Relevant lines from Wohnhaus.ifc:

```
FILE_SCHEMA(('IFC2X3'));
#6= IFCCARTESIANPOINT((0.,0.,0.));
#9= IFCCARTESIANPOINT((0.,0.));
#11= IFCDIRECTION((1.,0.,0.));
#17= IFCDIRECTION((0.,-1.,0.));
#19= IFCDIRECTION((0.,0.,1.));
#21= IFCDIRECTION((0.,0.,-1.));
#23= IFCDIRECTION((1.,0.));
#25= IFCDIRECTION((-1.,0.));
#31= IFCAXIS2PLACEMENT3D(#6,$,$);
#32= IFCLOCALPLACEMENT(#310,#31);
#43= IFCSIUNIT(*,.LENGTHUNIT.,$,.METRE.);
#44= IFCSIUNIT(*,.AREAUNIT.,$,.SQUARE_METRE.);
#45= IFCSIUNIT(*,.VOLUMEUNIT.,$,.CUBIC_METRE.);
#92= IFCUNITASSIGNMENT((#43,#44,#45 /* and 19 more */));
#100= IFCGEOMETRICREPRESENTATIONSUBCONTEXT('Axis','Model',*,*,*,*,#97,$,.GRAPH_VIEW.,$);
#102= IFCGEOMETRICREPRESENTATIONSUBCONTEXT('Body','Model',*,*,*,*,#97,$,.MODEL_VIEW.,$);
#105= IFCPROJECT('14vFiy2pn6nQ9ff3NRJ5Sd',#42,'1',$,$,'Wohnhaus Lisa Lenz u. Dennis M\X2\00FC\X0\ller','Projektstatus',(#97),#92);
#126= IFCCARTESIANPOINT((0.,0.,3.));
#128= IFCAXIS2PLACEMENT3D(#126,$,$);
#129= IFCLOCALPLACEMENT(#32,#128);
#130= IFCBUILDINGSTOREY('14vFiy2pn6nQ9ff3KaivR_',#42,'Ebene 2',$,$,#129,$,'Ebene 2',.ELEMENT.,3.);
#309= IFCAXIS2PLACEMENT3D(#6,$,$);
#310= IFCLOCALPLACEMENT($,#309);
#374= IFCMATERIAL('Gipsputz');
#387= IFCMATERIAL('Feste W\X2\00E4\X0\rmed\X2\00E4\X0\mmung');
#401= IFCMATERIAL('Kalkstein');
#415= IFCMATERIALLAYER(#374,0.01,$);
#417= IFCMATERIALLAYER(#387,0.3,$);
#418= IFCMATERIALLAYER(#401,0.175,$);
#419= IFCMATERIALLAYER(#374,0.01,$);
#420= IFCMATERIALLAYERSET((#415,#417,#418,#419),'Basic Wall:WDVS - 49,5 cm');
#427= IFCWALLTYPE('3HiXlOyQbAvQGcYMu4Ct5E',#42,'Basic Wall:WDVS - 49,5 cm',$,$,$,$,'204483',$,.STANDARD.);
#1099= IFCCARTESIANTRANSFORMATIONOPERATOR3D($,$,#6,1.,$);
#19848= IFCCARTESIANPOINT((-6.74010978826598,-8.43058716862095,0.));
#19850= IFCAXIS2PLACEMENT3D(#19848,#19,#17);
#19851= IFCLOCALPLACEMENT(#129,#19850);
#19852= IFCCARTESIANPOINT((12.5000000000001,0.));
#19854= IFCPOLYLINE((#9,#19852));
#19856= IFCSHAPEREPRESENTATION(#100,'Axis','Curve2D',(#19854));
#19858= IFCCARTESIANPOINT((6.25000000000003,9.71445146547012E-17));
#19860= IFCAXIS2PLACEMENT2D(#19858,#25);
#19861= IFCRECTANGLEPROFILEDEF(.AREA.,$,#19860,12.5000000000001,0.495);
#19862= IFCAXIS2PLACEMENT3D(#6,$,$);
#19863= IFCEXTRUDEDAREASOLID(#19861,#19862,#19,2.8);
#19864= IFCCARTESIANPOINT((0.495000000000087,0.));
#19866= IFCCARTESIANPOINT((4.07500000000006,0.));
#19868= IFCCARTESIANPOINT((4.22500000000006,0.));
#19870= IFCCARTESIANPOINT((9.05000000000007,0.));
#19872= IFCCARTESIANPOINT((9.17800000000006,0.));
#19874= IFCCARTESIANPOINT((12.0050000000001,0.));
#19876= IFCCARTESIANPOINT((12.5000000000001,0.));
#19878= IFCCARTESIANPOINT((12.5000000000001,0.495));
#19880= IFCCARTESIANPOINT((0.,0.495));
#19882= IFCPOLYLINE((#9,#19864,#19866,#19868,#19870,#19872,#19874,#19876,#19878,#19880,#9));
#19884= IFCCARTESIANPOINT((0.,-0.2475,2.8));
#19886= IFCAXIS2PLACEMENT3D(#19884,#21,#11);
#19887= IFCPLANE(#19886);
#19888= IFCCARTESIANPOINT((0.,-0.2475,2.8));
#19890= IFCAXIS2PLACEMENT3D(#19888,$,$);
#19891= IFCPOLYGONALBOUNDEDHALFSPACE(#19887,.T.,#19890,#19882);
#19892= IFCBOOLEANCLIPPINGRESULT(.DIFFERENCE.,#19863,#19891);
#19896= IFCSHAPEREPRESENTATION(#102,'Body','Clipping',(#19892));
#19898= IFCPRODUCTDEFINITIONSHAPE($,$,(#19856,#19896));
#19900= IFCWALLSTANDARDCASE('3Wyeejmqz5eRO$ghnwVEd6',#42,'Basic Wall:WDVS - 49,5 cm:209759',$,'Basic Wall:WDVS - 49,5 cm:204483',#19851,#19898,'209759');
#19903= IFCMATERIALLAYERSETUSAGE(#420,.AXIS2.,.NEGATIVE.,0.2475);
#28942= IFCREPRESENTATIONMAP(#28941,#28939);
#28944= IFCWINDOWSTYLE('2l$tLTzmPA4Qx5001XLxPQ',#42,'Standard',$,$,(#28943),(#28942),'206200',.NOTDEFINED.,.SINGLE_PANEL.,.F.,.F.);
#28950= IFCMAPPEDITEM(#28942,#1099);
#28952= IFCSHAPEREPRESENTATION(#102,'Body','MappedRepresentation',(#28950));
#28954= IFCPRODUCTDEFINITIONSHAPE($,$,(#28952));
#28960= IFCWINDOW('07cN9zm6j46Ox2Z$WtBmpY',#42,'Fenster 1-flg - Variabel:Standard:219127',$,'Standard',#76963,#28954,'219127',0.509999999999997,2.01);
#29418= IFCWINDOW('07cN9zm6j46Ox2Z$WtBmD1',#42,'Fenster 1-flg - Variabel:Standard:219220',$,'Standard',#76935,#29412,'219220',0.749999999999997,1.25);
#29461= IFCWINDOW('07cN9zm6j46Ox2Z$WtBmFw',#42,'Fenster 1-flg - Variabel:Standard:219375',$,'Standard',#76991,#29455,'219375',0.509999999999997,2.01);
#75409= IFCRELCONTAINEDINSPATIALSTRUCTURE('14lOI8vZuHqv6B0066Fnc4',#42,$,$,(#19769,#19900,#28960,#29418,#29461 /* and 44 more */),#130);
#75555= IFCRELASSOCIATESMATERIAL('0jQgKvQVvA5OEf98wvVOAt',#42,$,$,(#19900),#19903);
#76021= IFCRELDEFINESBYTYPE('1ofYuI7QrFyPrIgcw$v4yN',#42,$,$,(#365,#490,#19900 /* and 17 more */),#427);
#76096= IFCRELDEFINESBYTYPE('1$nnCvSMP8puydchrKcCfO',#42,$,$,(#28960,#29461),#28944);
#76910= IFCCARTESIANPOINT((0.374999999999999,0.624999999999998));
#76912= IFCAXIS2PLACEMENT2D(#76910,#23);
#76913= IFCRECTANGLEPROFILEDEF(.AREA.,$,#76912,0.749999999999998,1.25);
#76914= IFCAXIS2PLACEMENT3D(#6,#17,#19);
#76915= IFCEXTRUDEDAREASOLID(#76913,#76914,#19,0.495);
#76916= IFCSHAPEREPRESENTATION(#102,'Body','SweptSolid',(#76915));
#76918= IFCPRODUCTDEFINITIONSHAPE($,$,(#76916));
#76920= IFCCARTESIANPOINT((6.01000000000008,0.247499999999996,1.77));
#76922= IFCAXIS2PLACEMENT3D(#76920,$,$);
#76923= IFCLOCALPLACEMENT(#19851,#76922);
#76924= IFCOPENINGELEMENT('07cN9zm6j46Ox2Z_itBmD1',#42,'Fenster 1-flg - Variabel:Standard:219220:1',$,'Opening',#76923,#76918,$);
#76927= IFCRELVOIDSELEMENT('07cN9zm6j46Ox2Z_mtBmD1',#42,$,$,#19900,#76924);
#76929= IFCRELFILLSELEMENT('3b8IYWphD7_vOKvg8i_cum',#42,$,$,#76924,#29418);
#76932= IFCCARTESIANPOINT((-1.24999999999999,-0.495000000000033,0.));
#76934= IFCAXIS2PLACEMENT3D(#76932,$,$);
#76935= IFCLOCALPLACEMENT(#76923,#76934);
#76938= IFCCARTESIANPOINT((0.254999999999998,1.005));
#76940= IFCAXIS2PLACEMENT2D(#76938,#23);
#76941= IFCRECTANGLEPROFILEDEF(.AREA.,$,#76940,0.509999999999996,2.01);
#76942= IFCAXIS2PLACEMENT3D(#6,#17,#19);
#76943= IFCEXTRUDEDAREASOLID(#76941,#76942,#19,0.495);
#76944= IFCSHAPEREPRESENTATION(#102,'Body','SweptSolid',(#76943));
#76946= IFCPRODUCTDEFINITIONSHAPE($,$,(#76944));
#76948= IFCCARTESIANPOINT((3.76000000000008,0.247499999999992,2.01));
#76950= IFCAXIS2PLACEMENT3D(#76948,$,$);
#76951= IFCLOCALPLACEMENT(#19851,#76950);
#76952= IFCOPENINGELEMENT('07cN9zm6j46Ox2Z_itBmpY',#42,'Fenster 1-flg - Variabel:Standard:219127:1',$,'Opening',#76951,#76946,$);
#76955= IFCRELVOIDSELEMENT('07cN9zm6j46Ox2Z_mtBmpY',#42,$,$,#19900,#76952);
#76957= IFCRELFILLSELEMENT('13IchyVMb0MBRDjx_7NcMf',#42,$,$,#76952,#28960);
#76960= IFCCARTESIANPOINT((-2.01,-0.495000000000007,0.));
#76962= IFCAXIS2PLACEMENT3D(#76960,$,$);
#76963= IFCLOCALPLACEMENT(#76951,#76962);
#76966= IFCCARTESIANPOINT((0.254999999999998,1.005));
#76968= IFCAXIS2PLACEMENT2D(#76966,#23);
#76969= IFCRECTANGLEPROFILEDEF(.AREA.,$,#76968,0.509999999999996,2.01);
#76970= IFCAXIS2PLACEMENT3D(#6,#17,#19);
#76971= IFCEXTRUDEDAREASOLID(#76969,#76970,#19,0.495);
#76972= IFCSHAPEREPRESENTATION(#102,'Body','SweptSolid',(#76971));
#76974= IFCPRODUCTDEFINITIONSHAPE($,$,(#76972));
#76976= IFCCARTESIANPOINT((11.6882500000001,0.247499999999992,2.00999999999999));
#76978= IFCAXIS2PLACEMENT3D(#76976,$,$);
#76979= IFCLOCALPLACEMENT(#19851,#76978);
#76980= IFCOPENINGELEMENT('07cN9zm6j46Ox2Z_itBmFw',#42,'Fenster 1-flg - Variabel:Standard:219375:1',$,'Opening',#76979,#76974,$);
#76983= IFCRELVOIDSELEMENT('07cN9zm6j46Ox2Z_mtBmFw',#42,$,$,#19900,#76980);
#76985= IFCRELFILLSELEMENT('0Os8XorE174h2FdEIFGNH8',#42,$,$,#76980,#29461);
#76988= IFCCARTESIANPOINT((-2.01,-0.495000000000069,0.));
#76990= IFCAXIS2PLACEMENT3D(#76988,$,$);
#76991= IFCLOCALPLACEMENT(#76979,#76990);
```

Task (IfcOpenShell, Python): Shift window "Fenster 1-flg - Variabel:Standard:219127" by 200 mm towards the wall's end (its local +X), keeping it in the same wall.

```python
import ifcopenshell
import ifcopenshell.api.geometry
import ifcopenshell.util.placement
import ifcopenshell.util.unit

model = ifcopenshell.open("Wohnhaus.ifc")
unit_scale = ifcopenshell.util.unit.calculate_unit_scale(model)

window = model.by_id(28960)
opening = window.FillsVoids[0].RelatingOpeningElement
wall = opening.VoidsElements[0].RelatingBuildingElement

wall_matrix = ifcopenshell.util.placement.get_local_placement(wall.ObjectPlacement)
shift = wall_matrix[:3, 0] * 0.2 / unit_scale
before = ifcopenshell.util.placement.get_local_placement(window.ObjectPlacement)[:3, 3].copy()

# The window is placed relative to its opening, so it follows when the opening moves.
matrix = ifcopenshell.util.placement.get_local_placement(opening.ObjectPlacement)
matrix[:3, 3] += shift
ifcopenshell.api.geometry.edit_object_placement(
    model, product=opening, matrix=matrix, is_si=False, should_transform_children=True
)

after = ifcopenshell.util.placement.get_local_placement(window.ObjectPlacement)[:3, 3]
print("window moved by", (after - before).round(3) + 0.0)

model.write("Wohnhaus_rev.ifc")
```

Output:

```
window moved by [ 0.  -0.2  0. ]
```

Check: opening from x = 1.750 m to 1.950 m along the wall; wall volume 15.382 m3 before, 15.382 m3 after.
